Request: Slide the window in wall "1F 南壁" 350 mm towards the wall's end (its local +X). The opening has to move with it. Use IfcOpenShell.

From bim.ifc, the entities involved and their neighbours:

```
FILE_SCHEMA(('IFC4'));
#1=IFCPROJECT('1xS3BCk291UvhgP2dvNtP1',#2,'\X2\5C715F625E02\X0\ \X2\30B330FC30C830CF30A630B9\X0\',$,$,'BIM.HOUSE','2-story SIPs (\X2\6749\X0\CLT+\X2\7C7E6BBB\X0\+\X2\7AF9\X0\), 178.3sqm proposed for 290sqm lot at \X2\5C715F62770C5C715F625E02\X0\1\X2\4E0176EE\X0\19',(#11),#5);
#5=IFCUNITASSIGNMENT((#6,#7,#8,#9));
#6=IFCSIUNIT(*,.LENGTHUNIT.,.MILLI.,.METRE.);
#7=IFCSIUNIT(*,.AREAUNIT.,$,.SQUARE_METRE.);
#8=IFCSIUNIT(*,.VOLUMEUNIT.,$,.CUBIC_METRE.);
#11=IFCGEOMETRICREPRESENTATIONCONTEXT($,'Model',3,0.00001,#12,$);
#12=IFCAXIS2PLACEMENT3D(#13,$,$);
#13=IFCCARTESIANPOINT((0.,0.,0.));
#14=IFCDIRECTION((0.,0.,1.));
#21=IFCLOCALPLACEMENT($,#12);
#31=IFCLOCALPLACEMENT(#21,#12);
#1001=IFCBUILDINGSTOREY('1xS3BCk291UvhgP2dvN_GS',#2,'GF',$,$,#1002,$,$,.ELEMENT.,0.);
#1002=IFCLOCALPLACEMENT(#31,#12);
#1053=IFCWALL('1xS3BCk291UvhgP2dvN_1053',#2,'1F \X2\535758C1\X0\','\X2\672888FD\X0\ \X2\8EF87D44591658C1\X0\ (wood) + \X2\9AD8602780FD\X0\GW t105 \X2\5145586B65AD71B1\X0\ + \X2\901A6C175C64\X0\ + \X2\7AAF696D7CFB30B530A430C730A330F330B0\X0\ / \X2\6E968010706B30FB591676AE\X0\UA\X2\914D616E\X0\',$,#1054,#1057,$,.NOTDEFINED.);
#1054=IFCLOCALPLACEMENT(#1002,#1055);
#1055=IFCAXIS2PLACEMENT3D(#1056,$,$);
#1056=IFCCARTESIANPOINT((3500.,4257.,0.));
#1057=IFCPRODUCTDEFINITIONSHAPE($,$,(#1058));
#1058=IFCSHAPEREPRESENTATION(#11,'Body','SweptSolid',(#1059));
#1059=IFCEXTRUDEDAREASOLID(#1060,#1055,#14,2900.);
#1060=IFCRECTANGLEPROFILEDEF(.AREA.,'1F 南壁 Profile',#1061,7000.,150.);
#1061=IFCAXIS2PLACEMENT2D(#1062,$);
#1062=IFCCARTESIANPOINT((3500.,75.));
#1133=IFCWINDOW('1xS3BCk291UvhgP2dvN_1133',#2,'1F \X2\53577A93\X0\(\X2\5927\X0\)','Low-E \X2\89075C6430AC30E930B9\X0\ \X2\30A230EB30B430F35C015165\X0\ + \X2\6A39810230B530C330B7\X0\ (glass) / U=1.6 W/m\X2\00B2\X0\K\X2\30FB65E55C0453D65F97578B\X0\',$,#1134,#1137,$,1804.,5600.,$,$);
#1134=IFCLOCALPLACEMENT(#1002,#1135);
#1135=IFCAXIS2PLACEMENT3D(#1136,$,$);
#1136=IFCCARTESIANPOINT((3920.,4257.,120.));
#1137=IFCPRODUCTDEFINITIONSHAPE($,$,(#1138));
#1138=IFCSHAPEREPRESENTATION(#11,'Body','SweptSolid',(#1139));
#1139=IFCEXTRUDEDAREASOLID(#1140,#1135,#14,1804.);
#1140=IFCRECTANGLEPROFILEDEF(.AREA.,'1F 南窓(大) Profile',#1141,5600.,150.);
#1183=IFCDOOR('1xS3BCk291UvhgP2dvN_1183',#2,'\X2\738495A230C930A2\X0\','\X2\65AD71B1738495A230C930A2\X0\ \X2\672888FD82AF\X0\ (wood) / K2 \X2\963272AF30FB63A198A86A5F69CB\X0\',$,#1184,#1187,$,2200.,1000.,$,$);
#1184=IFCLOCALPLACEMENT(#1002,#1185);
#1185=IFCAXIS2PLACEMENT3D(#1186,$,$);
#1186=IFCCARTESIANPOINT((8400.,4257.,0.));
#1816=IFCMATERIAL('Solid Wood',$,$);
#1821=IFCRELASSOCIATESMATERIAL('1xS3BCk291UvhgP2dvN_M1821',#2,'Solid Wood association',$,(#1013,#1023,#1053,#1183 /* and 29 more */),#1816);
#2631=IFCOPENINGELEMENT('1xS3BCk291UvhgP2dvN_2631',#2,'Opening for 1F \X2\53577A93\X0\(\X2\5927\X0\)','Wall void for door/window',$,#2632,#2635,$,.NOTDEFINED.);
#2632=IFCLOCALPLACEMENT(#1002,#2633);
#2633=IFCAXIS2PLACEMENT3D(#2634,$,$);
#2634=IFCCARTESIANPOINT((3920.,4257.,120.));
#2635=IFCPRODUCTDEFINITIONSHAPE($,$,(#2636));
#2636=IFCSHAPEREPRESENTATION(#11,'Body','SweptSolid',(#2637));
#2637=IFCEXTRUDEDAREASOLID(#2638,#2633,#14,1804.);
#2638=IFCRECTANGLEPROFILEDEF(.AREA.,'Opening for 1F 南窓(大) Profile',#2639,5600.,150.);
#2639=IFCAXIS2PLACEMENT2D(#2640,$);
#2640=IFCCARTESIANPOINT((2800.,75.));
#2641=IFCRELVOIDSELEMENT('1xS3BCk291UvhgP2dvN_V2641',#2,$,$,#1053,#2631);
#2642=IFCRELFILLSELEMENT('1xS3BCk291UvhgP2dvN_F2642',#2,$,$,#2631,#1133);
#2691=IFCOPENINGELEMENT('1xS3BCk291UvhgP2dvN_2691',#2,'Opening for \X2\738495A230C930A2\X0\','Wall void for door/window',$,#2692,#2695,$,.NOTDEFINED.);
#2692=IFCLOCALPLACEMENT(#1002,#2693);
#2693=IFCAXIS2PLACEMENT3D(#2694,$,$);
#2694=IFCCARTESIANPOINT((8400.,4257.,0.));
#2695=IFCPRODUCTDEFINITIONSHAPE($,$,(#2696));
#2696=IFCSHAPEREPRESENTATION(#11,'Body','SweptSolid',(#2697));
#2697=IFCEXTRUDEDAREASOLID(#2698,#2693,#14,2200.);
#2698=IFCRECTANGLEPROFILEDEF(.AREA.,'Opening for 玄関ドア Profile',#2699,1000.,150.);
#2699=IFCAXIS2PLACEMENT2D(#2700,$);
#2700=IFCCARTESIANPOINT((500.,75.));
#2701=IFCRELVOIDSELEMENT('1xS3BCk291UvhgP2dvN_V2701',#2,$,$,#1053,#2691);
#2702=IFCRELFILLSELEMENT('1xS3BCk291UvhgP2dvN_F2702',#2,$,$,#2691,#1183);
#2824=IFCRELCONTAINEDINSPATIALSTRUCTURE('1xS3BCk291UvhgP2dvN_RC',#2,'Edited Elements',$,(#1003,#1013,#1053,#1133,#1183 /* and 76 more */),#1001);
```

```python
import ifcopenshell
import ifcopenshell.api.geometry
import ifcopenshell.util.placement
import ifcopenshell.util.unit

model = ifcopenshell.open("bim.ifc")
unit_scale = ifcopenshell.util.unit.calculate_unit_scale(model)

window = model.by_guid("1xS3BCk291UvhgP2dvN_1133")
opening = window.FillsVoids[0].RelatingOpeningElement
wall = opening.VoidsElements[0].RelatingBuildingElement

wall_matrix = ifcopenshell.util.placement.get_local_placement(wall.ObjectPlacement)
shift = wall_matrix[:3, 0] * 0.35 / unit_scale
before = ifcopenshell.util.placement.get_local_placement(window.ObjectPlacement)[:3, 3].copy()

# The window is not placed relative to its opening, so move both.
for product in (opening, window):
    matrix = ifcopenshell.util.placement.get_local_placement(product.ObjectPlacement)
    matrix[:3, 3] += shift
    ifcopenshell.api.geometry.edit_object_placement(model, product=product, matrix=matrix, is_si=False)

after = ifcopenshell.util.placement.get_local_placement(window.ObjectPlacement)[:3, 3]
print("window moved by", (after - before).round(3) + 0.0)

model.write("bim_rev.ifc")
```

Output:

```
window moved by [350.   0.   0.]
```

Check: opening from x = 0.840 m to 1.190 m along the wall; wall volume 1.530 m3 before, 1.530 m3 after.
